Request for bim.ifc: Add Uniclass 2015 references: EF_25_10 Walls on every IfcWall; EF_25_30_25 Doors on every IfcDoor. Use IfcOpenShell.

First a look at what the model holds.

```python
import ifcopenshell

model = ifcopenshell.open("bim.ifc")
print(model.schema)
print("classifications:", [c.Name for c in model.by_type("IfcClassification")])
for ifc_class in ("IfcDoor", "IfcRoof", "IfcStair", "IfcWall", "IfcWindow"):
    print(ifc_class, len(model.by_type(ifc_class)))
```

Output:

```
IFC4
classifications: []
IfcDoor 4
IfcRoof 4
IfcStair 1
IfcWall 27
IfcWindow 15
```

```python
import ifcopenshell
import ifcopenshell.api.classification

model = ifcopenshell.open("bim.ifc")

system = ifcopenshell.api.classification.add_classification(model, classification="Uniclass 2015")

codes = {
    "IfcWall": ("EF_25_10", "Walls"),
    "IfcDoor": ("EF_25_30_25", "Doors"),
}
for ifc_class, (code, name) in codes.items():
    products = model.by_type(ifc_class)
    ifcopenshell.api.classification.add_reference(
        model, products=products, classification=system, identification=code, name=name
    )
    print(code, len(products))

model.write("bim_rev.ifc")
```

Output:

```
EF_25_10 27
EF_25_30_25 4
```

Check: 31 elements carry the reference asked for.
